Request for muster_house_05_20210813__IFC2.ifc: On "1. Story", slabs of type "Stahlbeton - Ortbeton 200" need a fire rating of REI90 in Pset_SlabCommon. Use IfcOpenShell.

First a look at what the model holds.

```python
import ifcopenshell
import ifcopenshell.util.element

model = ifcopenshell.open("muster_house_05_20210813__IFC2.ifc")
print(model.schema)
storey = next(s for s in model.by_type("IfcBuildingStorey") if s.Name == "1. Story")
slabs = [e for e in ifcopenshell.util.element.get_decomposition(storey) if e.is_a("IfcSlab")]
seen = {}
for e in slabs:
    element_type = ifcopenshell.util.element.get_type(e)
    key = (element_type.Name if element_type != e and element_type else None, ifcopenshell.util.element.get_pset(e, "Pset_SlabCommon", "FireRating"))
    seen[key] = seen.get(key, 0) + 1
for (name, value), count in sorted(seen.items(), key=str):
    print(count, "x", name, "|", value)
```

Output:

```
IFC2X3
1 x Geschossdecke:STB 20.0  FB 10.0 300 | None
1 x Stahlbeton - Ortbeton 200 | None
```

```python
import ifcopenshell
import ifcopenshell.api.pset
import ifcopenshell.util.element

model = ifcopenshell.open("muster_house_05_20210813__IFC2.ifc")

storey = next(s for s in model.by_type("IfcBuildingStorey") if s.Name == "1. Story")
slabs = [e for e in ifcopenshell.util.element.get_decomposition(storey) if e.is_a("IfcSlab")]

count = 0
for e in slabs:
    element_type = ifcopenshell.util.element.get_type(e)
    if element_type in (None, e) or element_type.Name != "Stahlbeton - Ortbeton 200":
        continue
    # add_pset returns the element's existing set when there is one.
    pset = ifcopenshell.api.pset.add_pset(model, product=e, name="Pset_SlabCommon")
    ifcopenshell.api.pset.edit_pset(model, pset=pset, properties={"FireRating": "REI90"})
    count += 1

print(count, "slabs updated")

model.write("muster_house_05_20210813__IFC2_v2.ifc")
```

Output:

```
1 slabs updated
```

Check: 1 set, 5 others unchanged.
